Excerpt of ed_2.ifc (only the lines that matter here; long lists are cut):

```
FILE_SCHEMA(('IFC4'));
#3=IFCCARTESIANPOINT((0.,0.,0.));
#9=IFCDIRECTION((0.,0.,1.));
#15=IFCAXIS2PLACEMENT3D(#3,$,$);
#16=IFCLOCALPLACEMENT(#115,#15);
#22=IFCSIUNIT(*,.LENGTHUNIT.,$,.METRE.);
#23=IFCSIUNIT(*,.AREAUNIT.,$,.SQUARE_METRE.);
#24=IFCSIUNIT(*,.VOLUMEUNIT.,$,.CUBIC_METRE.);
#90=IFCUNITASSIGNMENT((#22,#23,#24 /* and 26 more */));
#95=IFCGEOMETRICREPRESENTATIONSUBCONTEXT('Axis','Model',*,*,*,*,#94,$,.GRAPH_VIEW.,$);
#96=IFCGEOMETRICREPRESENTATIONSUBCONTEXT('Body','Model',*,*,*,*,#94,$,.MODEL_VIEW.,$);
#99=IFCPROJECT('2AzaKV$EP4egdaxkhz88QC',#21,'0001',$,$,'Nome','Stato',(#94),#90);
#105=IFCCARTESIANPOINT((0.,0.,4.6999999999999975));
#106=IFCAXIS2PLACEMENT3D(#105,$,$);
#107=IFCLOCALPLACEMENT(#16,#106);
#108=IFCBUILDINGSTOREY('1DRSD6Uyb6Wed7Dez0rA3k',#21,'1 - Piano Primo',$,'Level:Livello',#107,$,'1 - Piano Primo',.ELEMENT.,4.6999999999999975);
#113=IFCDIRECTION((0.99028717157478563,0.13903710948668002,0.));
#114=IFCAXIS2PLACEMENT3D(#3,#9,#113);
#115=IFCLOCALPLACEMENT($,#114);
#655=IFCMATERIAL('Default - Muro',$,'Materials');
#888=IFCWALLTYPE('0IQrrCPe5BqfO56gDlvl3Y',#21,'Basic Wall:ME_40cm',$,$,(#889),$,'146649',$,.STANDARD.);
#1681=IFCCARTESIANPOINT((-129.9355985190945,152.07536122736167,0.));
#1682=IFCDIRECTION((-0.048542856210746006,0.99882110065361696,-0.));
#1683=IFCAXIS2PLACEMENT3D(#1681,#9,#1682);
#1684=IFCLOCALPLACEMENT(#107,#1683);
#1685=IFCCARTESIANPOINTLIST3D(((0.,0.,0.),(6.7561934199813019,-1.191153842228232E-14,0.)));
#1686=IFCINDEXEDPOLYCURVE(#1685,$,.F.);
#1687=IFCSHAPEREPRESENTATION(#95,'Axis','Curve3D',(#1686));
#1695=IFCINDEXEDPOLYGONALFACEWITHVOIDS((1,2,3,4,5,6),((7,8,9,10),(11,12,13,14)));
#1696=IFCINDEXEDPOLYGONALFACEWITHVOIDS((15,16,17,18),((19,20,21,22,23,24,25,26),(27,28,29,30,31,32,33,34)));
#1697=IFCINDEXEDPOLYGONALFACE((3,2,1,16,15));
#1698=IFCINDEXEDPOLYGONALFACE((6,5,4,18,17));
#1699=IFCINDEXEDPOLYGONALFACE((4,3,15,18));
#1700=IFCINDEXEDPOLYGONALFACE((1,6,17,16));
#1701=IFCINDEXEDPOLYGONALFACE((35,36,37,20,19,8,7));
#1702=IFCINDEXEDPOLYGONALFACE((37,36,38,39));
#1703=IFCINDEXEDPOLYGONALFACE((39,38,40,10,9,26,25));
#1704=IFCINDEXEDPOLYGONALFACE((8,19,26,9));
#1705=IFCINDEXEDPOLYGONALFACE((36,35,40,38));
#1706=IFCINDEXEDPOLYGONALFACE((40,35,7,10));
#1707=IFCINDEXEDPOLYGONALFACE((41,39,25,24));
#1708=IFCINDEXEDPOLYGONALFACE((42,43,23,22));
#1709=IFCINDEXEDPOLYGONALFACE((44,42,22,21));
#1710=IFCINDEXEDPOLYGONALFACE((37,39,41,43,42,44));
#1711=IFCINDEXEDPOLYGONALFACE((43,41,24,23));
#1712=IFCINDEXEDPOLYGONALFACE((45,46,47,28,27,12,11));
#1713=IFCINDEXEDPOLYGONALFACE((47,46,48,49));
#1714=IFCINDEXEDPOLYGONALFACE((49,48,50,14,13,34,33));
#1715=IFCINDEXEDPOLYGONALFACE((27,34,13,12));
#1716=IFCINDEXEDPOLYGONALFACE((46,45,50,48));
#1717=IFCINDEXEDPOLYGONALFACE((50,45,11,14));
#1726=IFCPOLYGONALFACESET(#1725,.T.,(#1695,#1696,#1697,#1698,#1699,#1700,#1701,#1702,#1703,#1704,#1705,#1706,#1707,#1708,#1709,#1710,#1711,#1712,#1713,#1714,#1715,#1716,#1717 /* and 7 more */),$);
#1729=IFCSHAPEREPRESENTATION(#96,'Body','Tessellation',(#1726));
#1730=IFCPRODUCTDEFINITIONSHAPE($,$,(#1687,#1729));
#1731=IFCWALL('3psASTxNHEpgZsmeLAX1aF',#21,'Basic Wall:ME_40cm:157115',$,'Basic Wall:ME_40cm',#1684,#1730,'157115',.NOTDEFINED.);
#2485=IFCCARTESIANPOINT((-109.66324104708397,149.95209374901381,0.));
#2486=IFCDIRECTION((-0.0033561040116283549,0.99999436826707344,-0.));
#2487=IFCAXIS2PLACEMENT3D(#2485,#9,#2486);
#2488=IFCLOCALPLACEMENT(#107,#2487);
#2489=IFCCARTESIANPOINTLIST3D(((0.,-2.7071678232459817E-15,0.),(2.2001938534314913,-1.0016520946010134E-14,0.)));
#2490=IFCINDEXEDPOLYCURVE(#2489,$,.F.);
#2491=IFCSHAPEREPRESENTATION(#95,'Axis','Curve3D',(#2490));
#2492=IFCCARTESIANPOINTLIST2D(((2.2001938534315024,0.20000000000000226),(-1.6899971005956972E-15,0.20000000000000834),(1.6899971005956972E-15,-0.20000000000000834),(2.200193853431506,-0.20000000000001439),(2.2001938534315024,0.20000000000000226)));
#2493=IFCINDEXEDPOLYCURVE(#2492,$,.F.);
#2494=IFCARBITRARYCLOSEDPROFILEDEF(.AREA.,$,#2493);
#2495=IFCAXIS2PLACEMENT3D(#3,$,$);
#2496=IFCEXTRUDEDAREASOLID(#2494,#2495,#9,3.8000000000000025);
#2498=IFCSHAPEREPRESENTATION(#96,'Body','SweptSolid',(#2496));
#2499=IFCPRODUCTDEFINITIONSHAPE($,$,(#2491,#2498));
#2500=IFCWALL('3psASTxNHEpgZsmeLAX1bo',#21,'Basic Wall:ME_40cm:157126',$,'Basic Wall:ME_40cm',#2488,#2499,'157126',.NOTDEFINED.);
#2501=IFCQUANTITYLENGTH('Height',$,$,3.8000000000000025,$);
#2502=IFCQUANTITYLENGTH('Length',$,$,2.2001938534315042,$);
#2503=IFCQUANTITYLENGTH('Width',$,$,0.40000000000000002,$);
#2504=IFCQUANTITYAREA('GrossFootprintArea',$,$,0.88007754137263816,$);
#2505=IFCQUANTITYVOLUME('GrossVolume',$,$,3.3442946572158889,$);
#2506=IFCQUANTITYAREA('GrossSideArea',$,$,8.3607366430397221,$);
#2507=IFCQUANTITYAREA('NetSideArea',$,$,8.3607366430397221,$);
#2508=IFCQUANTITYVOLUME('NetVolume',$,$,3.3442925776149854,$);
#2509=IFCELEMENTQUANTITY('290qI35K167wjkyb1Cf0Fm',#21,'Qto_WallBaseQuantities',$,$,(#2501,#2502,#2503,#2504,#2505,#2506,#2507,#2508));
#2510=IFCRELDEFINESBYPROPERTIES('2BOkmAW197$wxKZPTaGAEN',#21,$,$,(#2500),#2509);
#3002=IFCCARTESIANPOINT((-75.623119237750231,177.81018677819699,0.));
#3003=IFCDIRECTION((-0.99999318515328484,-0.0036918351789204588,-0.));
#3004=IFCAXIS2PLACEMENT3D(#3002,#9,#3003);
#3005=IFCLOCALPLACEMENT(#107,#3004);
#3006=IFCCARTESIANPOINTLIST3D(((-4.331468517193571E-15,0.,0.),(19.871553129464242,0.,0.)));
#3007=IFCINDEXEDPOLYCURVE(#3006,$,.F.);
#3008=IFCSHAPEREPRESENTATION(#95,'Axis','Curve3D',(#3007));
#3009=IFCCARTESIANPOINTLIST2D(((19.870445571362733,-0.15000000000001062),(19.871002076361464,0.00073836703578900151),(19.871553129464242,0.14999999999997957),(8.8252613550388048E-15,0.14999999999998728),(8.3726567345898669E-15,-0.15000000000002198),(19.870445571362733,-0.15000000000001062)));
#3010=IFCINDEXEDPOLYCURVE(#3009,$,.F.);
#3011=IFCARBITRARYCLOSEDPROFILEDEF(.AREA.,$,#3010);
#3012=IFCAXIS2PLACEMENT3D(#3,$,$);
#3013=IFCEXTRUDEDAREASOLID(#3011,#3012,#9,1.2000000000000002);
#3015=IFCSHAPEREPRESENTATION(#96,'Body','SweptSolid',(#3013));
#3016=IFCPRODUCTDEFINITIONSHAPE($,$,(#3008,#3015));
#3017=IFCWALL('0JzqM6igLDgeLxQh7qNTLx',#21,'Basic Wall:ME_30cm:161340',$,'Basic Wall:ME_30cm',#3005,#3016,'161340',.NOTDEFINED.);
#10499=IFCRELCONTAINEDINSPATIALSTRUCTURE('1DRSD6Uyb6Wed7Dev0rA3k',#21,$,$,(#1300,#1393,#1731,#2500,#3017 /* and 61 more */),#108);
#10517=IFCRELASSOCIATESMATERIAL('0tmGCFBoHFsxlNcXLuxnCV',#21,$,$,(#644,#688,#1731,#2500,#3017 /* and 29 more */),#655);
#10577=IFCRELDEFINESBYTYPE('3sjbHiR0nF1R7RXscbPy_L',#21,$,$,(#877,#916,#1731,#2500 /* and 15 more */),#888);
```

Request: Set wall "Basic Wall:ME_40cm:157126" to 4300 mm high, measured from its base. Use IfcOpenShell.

```python
import ifcopenshell
import ifcopenshell.api.pset
import ifcopenshell.geom
import ifcopenshell.util.element
import ifcopenshell.util.representation
import ifcopenshell.util.shape
import ifcopenshell.util.unit

model = ifcopenshell.open("ed_2.ifc")
unit_scale = ifcopenshell.util.unit.calculate_unit_scale(model)
area_scale = ifcopenshell.util.unit.calculate_unit_scale(model, "AREAUNIT")
volume_scale = ifcopenshell.util.unit.calculate_unit_scale(model, "VOLUMEUNIT")
settings = ifcopenshell.geom.settings()


def volume(element):
    """Net volume in cubic metres, openings subtracted."""
    shape = ifcopenshell.geom.create_shape(settings, element)
    return ifcopenshell.util.shape.get_volume(shape.geometry)


wall = model.by_guid("3psASTxNHEpgZsmeLAX1bo")
before = volume(wall)

body = ifcopenshell.util.representation.get_representation(wall, "Model", "Body")
solid = body.Items[0]
old_height = solid.Depth
solid.Depth = 4.3 / unit_scale
after = volume(wall)
thickness = 0.4  # wall thickness in metres

# Update the stored height, areas and volumes.
qto = model.by_id(ifcopenshell.util.element.get_pset(wall, "Qto_WallBaseQuantities", should_inherit=False)["id"])
ifcopenshell.api.pset.edit_qto(model, qto=qto, properties={
    "Height": solid.Depth,
    "GrossVolume": ifcopenshell.util.element.get_pset(wall, "Qto_WallBaseQuantities", "GrossVolume") * solid.Depth / old_height,
    "GrossSideArea": ifcopenshell.util.element.get_pset(wall, "Qto_WallBaseQuantities", "GrossSideArea") * solid.Depth / old_height,
    "NetSideArea": after / thickness / area_scale,
    "NetVolume": after / volume_scale,
})

print(f"height {old_height:g} -> {solid.Depth:g}, volume {before:.3f} -> {after:.3f} m3")

model.write("ed_2-out.ifc")
```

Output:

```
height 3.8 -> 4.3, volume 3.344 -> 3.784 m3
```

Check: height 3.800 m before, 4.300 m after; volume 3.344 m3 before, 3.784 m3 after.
